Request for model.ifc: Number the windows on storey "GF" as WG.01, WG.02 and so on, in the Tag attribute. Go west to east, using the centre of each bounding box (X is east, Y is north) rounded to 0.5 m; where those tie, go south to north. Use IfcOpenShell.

First a look at what the model holds.

```python
import ifcopenshell
import ifcopenshell.util.element
import ifcopenshell.util.placement

model = ifcopenshell.open("model.ifc")
print(model.schema)
storey = next(s for s in model.by_type("IfcBuildingStorey") if s.Name == "GF")
windows = [e for e in ifcopenshell.util.element.get_decomposition(storey) if e.is_a("IfcWindow")]
for e in sorted(windows, key=lambda e: e.id()):
    origin = ifcopenshell.util.placement.get_local_placement(e.ObjectPlacement)[:3, 3]
    print(e.id(), e.Tag, e.Name, origin.round(2) + 0.0, sep=" | ")
```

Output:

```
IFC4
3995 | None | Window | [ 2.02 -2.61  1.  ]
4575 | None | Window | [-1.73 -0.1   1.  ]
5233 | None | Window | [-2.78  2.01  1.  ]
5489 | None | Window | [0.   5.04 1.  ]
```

```python
import ifcopenshell
import ifcopenshell.geom
import ifcopenshell.util.element
import ifcopenshell.util.shape

model = ifcopenshell.open("model.ifc")
settings = ifcopenshell.geom.settings()
settings.set("use-world-coords", True)


def centre(element):
    shape = ifcopenshell.geom.create_shape(settings, element)
    return ifcopenshell.util.shape.get_bbox_centroid(shape.geometry)


storey = next(s for s in model.by_type("IfcBuildingStorey") if s.Name == "GF")
windows = [e for e in ifcopenshell.util.element.get_decomposition(storey) if e.is_a("IfcWindow")]

# Insertion points can sit at a corner or the storey origin, so sort by the geometry (in metres).
centres = {e: centre(e) for e in windows}
windows.sort(key=lambda e: (round(centres[e][0] / 0.5), centres[e][1]))

for i, e in enumerate(windows, start=1):
    number = f"WG.{i:02d}"
    e.Tag = number
    print(e.id(), number)

model.write("model_edited.ifc")
```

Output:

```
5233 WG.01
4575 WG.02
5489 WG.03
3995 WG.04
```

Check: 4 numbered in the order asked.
